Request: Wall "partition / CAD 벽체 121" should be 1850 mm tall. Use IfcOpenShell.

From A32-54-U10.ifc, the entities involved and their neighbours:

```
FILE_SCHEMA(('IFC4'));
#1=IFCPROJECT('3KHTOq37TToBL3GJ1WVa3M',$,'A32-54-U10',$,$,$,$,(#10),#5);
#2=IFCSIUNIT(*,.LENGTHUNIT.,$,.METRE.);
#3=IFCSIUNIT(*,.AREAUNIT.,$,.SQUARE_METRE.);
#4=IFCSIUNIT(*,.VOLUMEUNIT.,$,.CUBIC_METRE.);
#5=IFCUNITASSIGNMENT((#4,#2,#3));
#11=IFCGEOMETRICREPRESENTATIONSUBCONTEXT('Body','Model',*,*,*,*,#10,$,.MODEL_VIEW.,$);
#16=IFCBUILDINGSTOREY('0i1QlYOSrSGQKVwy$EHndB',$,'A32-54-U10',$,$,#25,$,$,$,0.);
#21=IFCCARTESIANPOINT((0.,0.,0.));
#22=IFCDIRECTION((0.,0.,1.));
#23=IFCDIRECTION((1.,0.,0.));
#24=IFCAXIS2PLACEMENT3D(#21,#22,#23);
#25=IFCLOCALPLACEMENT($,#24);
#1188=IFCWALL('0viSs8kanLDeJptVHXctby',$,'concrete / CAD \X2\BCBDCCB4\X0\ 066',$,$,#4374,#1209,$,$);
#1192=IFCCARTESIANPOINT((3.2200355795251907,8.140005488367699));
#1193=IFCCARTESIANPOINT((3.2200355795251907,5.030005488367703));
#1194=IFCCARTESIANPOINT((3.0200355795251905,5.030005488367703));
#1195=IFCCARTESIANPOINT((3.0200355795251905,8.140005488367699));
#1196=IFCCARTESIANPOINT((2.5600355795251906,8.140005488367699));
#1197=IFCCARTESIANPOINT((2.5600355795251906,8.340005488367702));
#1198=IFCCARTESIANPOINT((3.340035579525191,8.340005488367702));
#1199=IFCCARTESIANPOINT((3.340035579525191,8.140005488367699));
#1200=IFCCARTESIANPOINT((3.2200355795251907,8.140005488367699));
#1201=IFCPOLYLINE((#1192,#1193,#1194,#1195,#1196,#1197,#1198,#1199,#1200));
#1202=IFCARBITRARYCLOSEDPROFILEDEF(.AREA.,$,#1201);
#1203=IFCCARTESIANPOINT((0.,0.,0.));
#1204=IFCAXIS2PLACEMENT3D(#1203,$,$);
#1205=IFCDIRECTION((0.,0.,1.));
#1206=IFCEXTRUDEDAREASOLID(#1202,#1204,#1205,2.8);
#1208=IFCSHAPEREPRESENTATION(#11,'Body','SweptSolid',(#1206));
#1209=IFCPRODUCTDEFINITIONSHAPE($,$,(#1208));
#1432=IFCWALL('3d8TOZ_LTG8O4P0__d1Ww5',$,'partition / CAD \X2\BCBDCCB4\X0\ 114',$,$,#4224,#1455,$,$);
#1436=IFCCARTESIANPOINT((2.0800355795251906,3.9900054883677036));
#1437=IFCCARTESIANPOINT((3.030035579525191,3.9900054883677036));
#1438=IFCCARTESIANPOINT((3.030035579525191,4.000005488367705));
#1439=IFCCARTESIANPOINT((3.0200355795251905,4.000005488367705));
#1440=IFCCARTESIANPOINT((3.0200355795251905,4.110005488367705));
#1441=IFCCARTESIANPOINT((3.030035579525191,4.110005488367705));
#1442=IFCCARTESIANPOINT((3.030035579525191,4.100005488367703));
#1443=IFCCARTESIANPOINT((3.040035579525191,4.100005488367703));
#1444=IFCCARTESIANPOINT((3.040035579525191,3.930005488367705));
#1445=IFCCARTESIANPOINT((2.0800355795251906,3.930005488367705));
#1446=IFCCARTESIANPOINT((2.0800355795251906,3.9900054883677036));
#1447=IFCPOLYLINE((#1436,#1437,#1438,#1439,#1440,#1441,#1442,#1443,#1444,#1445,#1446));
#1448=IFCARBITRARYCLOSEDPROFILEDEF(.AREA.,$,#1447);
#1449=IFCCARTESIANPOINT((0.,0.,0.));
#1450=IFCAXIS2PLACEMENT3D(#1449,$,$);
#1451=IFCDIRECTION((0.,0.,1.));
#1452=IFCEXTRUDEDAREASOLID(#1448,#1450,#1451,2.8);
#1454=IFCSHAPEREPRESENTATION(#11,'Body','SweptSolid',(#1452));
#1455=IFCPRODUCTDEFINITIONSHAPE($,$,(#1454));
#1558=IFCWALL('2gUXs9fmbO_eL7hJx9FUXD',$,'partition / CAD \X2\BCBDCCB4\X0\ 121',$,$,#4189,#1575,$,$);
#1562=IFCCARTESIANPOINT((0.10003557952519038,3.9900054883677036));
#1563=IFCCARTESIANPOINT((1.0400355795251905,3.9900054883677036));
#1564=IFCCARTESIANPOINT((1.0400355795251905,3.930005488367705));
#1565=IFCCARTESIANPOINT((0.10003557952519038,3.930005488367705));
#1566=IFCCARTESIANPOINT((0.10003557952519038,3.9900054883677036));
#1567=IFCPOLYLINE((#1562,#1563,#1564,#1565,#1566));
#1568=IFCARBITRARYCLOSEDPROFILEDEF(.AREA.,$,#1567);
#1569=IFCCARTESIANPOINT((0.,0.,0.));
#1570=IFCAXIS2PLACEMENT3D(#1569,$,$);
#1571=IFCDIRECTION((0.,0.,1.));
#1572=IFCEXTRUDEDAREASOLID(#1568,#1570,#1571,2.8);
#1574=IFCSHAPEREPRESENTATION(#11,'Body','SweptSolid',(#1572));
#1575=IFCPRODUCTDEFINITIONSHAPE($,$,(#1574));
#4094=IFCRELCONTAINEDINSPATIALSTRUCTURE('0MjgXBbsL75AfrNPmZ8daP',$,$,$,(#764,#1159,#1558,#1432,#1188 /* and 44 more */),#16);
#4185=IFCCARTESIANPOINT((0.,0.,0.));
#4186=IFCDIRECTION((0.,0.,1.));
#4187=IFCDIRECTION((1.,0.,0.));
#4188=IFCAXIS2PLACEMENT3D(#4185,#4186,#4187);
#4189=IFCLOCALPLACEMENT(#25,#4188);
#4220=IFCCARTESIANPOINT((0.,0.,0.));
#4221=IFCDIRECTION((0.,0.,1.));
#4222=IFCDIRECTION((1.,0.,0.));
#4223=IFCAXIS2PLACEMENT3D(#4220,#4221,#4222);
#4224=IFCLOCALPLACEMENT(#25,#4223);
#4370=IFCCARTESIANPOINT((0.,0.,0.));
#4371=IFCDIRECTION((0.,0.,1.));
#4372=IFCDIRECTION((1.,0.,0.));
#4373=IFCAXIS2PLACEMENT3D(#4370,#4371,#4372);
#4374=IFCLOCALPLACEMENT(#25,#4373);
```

```python
import ifcopenshell
import ifcopenshell.geom
import ifcopenshell.util.representation
import ifcopenshell.util.shape

model = ifcopenshell.open("A32-54-U10.ifc")
settings = ifcopenshell.geom.settings()


def volume(element):
    """Net volume in cubic metres, openings subtracted."""
    shape = ifcopenshell.geom.create_shape(settings, element)
    return ifcopenshell.util.shape.get_volume(shape.geometry)


wall = model.by_guid("2gUXs9fmbO_eL7hJx9FUXD")
before = volume(wall)

body = ifcopenshell.util.representation.get_representation(wall, "Model", "Body")
solid = body.Items[0]
old_height = solid.Depth
solid.Depth = 1.85
after = volume(wall)

print(f"height {old_height:g} -> {solid.Depth:g}, volume {before:.3f} -> {after:.3f} m3")

model.write("A32-54-U10_edited.ifc")
```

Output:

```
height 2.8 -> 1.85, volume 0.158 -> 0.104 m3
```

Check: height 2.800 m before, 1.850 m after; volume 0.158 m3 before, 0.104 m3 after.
